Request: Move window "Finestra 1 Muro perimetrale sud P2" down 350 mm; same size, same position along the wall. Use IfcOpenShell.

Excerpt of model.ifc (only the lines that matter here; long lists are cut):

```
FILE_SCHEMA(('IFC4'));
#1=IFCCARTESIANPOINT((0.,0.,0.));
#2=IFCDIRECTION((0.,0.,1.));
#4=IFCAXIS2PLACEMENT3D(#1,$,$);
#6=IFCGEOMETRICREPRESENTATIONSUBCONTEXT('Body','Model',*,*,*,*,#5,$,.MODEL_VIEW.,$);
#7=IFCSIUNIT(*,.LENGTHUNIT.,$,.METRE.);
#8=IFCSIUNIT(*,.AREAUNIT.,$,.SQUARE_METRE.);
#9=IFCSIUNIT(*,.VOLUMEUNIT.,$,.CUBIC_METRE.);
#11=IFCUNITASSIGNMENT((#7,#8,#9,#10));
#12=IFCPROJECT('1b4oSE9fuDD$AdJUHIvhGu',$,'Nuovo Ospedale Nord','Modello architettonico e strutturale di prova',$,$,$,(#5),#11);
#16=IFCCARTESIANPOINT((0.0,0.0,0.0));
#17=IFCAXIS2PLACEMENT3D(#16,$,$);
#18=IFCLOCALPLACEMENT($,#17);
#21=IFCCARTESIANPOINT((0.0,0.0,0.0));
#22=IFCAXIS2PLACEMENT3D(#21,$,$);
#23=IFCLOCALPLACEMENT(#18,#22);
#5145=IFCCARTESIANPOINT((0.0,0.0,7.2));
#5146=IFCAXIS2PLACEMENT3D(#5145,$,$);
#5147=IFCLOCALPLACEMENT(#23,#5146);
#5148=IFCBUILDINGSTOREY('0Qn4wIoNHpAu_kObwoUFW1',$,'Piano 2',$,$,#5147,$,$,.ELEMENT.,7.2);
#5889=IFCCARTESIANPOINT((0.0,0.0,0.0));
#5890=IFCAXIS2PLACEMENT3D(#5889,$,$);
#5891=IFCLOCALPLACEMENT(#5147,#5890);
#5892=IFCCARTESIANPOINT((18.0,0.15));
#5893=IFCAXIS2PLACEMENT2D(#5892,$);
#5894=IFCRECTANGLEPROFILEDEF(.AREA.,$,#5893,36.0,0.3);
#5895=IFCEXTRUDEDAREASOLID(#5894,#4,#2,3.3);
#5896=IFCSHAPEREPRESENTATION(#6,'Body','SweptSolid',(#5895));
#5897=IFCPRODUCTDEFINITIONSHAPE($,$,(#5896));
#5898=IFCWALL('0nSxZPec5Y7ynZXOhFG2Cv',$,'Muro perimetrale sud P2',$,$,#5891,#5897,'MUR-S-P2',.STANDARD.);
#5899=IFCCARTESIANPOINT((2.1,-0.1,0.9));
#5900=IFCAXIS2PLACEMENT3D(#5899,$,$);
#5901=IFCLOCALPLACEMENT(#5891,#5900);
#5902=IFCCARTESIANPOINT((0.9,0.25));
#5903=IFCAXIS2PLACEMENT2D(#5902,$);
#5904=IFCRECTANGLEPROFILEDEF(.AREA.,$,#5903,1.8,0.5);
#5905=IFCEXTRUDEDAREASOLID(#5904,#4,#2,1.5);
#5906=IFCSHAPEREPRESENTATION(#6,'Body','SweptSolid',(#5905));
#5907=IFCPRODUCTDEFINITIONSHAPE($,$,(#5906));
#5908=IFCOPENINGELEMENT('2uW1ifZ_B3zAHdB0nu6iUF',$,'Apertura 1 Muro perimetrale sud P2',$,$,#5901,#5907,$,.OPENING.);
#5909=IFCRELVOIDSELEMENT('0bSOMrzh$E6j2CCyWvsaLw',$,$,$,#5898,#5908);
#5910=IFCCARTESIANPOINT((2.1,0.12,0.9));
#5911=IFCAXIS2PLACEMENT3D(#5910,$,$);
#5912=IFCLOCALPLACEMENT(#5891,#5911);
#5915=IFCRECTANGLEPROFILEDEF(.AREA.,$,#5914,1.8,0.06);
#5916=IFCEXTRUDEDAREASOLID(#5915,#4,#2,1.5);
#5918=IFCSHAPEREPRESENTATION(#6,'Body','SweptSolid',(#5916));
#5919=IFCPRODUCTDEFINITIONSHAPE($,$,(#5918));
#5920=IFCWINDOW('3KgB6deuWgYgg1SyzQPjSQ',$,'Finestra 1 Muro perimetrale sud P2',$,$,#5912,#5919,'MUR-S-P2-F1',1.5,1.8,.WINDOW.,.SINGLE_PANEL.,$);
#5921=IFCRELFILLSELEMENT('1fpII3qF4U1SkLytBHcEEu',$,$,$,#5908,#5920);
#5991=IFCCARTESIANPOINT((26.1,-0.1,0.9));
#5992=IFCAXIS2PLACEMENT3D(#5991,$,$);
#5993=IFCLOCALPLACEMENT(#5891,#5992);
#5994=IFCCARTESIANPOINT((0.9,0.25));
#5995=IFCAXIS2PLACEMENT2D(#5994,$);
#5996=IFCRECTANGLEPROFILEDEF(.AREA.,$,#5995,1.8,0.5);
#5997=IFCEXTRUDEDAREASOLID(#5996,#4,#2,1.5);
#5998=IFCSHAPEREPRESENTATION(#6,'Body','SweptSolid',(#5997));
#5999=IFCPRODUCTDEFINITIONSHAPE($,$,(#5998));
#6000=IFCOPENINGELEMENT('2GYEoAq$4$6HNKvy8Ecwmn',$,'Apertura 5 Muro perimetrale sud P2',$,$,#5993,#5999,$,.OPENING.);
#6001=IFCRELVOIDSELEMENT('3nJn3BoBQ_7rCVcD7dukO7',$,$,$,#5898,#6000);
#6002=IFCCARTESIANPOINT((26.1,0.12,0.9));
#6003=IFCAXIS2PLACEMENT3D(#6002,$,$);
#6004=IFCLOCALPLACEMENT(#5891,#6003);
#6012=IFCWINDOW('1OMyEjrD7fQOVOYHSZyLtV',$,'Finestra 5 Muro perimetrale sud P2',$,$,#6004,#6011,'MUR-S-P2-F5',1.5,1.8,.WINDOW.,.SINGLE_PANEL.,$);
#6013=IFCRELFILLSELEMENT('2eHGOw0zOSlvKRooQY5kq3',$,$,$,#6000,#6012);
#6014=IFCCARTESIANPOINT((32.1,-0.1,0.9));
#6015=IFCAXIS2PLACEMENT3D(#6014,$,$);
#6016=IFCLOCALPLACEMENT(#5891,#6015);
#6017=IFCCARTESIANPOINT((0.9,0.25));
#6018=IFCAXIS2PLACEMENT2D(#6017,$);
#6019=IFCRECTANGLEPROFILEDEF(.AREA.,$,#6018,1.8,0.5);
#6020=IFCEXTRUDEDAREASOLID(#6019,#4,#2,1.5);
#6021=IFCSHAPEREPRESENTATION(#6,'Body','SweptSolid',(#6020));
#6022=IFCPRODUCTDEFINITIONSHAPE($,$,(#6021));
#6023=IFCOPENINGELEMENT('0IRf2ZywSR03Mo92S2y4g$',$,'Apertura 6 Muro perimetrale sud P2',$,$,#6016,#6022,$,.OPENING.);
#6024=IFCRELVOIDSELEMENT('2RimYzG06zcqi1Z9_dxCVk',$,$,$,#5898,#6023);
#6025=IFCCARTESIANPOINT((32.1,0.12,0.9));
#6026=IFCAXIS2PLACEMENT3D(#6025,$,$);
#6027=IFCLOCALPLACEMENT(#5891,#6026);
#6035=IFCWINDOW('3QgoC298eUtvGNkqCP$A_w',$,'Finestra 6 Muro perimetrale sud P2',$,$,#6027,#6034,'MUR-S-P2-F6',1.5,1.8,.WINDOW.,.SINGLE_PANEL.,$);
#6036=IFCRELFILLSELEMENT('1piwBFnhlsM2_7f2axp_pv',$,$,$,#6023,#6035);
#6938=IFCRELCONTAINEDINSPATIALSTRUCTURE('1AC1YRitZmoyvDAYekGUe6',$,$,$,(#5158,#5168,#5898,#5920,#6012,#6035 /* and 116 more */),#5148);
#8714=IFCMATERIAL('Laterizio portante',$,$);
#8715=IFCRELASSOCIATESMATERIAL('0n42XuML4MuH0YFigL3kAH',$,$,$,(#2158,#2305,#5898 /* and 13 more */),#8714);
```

```python
import numpy as np
import ifcopenshell
import ifcopenshell.api.geometry
import ifcopenshell.util.placement
import ifcopenshell.util.unit

model = ifcopenshell.open("model.ifc")
unit_scale = ifcopenshell.util.unit.calculate_unit_scale(model)

window = model.by_guid("3KgB6deuWgYgg1SyzQPjSQ")
opening = window.FillsVoids[0].RelatingOpeningElement
dz = -0.35 / unit_scale

shift = np.array([0.0, 0.0, dz])
# The window is not placed relative to its opening, so move both.
for product in (opening, window):
    matrix = ifcopenshell.util.placement.get_local_placement(product.ObjectPlacement)
    matrix[:3, 3] += shift
    ifcopenshell.api.geometry.edit_object_placement(model, product=product, matrix=matrix, is_si=False)

print(f"moved by {dz * unit_scale:+.3f} m")

model.write("model_rev.ifc")
```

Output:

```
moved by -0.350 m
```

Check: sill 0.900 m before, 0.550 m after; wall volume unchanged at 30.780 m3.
